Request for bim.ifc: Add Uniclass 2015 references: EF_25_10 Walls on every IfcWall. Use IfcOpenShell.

First a look at what the model holds.

```python
import ifcopenshell

model = ifcopenshell.open("bim.ifc")
print(model.schema)
print("classifications:", [c.Name for c in model.by_type("IfcClassification")])
for ifc_class in ("IfcDoor", "IfcRoof", "IfcStair", "IfcWall", "IfcWindow"):
    print(ifc_class, len(model.by_type(ifc_class)))
```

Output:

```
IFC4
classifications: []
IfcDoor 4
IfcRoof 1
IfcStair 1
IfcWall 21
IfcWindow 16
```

```python
import ifcopenshell
import ifcopenshell.api.classification

model = ifcopenshell.open("bim.ifc")

system = ifcopenshell.api.classification.add_classification(model, classification="Uniclass 2015")

codes = {
    "IfcWall": ("EF_25_10", "Walls"),
}
for ifc_class, (code, name) in codes.items():
    products = model.by_type(ifc_class)
    ifcopenshell.api.classification.add_reference(
        model, products=products, classification=system, identification=code, name=name
    )
    print(code, len(products))

model.write("bim_v2.ifc")
```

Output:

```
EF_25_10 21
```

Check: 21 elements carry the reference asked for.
